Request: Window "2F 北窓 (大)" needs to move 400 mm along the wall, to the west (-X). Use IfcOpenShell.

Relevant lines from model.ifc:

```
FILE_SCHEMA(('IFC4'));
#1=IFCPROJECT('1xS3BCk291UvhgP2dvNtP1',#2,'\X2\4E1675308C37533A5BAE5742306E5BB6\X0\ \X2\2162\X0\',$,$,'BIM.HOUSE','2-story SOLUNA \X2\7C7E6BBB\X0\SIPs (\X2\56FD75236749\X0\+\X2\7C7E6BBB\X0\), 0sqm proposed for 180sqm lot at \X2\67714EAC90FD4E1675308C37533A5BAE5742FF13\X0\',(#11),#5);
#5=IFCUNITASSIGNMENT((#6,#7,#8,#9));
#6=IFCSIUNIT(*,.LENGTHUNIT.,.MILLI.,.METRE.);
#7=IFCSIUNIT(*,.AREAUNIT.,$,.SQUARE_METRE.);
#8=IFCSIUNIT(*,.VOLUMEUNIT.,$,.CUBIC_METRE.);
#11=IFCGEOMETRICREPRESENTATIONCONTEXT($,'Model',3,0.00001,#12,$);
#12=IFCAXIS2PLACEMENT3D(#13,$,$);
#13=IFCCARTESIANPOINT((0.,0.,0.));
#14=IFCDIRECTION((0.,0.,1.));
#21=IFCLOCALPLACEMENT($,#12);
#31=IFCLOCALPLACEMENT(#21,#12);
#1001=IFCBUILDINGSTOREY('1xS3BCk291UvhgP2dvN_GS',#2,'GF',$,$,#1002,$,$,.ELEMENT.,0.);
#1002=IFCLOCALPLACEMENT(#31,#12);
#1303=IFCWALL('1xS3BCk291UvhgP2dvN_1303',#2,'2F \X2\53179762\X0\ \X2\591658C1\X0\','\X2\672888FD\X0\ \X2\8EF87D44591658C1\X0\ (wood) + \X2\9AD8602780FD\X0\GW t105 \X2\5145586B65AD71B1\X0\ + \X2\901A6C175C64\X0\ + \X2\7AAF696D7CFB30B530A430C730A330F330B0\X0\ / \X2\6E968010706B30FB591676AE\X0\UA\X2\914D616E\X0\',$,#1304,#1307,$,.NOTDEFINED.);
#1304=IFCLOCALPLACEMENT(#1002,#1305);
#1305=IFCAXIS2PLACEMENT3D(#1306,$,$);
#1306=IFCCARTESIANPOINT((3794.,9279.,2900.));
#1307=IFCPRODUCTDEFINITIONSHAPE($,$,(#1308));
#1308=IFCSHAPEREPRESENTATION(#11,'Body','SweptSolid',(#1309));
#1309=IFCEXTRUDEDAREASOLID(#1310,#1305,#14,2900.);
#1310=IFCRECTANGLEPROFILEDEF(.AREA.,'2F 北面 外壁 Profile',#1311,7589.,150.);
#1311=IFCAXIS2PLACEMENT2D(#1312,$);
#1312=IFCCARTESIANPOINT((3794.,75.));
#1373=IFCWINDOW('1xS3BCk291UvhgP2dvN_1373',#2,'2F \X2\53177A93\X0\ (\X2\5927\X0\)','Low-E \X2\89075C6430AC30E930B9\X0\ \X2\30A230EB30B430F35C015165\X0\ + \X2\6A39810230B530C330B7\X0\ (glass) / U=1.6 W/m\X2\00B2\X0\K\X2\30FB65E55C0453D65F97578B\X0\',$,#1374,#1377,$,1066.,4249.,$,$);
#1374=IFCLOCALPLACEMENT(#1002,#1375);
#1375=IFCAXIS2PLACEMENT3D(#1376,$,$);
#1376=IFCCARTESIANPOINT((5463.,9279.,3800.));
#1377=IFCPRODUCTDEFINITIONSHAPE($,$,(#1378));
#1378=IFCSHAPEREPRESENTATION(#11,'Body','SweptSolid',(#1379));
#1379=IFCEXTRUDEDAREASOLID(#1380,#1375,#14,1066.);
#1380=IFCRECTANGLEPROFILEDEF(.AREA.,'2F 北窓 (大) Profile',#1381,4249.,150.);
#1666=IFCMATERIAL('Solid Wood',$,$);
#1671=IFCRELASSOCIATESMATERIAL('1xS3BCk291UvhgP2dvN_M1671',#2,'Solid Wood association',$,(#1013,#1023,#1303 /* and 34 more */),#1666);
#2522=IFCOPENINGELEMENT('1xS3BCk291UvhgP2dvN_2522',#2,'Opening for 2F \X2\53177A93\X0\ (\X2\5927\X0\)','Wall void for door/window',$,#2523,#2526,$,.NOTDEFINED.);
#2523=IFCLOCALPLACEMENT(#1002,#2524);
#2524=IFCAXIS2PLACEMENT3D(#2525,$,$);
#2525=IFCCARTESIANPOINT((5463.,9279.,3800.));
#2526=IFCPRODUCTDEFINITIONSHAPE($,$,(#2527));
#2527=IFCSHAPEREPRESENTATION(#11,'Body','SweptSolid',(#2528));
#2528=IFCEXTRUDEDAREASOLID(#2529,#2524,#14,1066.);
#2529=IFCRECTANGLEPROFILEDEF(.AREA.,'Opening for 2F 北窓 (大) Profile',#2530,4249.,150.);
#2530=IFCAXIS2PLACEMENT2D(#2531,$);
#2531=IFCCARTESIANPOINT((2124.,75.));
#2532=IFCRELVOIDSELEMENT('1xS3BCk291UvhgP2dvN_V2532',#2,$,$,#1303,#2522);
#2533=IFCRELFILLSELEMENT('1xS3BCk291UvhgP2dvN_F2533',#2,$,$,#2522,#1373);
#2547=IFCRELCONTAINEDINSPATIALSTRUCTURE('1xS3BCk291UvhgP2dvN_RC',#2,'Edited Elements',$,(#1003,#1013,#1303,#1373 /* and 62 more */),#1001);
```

```python
import ifcopenshell
import ifcopenshell.api.geometry
import ifcopenshell.util.placement

model = ifcopenshell.open("model.ifc")

window = model.by_id(1373)
opening = window.FillsVoids[0].RelatingOpeningElement
wall = opening.VoidsElements[0].RelatingBuildingElement

wall_matrix = ifcopenshell.util.placement.get_local_placement(wall.ObjectPlacement)
shift = wall_matrix[:3, 0] * -400.0
before = ifcopenshell.util.placement.get_local_placement(window.ObjectPlacement)[:3, 3].copy()

# The window is not placed relative to its opening, so move both.
for product in (opening, window):
    matrix = ifcopenshell.util.placement.get_local_placement(product.ObjectPlacement)
    matrix[:3, 3] += shift
    ifcopenshell.api.geometry.edit_object_placement(model, product=product, matrix=matrix, is_si=False)

after = ifcopenshell.util.placement.get_local_placement(window.ObjectPlacement)[:3, 3]
print("window moved by", (after - before).round(3) + 0.0)

model.write("model_edited.ifc")
```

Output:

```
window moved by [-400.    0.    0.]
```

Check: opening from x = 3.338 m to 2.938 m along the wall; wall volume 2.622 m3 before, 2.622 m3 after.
